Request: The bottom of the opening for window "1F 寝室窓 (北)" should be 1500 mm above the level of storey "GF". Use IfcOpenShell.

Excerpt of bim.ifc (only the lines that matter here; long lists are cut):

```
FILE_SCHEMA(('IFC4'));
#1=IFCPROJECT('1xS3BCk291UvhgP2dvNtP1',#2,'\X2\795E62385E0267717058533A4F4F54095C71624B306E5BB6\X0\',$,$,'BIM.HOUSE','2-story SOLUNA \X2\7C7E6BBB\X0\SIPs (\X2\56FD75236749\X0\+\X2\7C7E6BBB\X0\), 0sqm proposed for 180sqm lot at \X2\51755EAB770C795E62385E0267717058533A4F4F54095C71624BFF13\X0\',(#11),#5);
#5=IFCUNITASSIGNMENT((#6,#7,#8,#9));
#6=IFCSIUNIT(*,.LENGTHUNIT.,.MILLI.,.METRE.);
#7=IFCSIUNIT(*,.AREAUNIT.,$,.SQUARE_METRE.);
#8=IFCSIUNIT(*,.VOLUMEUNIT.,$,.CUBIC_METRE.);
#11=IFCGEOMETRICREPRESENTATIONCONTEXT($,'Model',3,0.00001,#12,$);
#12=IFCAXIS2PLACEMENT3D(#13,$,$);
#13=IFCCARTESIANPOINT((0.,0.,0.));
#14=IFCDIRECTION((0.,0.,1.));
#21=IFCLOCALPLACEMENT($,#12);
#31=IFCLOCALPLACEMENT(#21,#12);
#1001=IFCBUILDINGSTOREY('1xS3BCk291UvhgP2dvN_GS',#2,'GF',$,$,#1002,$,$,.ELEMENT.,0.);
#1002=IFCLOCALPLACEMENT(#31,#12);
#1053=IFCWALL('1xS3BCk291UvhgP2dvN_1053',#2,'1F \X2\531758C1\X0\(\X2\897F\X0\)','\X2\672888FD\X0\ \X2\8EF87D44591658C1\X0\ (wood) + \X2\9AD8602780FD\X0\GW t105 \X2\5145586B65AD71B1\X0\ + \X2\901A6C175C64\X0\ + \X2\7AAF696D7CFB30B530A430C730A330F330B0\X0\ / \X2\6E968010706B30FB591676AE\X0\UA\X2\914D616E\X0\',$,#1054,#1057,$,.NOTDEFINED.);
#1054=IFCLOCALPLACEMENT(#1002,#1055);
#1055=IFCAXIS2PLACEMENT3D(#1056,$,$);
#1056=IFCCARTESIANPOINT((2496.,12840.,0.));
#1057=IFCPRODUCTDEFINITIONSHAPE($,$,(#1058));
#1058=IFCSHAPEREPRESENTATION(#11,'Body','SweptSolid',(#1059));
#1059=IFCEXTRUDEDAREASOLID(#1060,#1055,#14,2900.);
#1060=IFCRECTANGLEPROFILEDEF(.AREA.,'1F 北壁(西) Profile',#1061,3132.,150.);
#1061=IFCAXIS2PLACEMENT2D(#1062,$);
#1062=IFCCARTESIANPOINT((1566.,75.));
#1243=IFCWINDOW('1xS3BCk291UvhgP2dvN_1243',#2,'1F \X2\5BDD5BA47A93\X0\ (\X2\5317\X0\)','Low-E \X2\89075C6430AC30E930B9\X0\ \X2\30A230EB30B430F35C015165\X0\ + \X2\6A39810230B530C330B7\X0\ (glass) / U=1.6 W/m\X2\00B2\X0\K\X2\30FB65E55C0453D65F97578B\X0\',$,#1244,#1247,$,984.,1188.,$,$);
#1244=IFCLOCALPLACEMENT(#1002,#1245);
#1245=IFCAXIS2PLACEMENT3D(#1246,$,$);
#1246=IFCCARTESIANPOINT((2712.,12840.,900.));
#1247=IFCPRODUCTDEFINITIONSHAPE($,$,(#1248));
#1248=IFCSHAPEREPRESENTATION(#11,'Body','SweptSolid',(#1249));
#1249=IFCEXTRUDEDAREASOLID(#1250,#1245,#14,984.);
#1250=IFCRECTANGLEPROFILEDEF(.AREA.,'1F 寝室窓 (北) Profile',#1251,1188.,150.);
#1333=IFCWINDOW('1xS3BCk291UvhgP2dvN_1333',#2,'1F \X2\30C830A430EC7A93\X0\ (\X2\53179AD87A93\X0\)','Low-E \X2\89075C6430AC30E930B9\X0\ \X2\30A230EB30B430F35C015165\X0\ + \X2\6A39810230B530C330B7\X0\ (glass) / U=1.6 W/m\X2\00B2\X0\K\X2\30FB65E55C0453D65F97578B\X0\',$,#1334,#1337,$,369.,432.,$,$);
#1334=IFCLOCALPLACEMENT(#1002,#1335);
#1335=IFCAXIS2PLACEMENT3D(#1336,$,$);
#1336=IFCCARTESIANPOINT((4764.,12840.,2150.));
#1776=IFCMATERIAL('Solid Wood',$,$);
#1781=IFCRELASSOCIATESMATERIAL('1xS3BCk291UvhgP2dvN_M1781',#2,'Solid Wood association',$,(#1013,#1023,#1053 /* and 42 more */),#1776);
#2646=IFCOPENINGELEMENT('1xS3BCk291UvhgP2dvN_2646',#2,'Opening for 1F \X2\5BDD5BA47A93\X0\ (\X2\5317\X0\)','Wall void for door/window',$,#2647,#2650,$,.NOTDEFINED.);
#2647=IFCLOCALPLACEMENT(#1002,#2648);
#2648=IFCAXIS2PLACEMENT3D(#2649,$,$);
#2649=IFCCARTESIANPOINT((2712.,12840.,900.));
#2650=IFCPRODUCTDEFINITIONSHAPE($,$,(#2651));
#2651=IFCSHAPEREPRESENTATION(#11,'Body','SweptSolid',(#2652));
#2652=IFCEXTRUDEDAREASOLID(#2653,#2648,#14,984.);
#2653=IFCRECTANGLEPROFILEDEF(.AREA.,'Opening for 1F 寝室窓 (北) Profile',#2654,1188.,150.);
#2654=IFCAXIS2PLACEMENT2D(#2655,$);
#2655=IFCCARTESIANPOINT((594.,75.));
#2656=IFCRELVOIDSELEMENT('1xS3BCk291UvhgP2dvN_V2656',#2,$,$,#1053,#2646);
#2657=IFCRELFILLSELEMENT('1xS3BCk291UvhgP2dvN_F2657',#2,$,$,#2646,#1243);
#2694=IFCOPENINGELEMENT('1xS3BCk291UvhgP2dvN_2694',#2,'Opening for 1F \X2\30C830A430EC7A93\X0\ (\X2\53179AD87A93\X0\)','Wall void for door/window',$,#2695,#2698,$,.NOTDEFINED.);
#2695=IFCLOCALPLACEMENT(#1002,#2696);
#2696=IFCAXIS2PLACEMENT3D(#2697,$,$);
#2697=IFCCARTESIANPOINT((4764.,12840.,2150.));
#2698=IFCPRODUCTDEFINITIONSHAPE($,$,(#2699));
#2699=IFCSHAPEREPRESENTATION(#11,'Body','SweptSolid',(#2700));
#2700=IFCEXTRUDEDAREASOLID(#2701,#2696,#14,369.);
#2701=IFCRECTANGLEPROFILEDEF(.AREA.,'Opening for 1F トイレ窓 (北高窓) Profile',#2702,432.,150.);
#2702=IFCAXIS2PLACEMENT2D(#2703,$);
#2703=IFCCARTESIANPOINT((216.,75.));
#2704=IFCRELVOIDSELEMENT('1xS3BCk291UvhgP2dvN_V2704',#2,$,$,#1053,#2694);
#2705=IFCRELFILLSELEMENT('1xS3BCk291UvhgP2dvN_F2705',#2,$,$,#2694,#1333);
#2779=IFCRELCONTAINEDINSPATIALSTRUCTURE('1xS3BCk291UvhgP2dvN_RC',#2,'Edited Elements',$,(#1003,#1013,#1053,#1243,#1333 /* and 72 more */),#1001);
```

```python
import numpy as np
import ifcopenshell
import ifcopenshell.api.geometry
import ifcopenshell.geom
import ifcopenshell.util.element
import ifcopenshell.util.placement
import ifcopenshell.util.shape
import ifcopenshell.util.unit

model = ifcopenshell.open("bim.ifc")
unit_scale = ifcopenshell.util.unit.calculate_unit_scale(model)

window = model.by_guid("1xS3BCk291UvhgP2dvN_1243")
opening = window.FillsVoids[0].RelatingOpeningElement
storey = ifcopenshell.util.element.get_container(window, ifc_class="IfcBuildingStorey")
level = ifcopenshell.util.placement.get_local_placement(storey.ObjectPlacement)[2, 3]

# The opening's origin need not be at the sill, so measure its lowest point.
shape = ifcopenshell.geom.create_shape(ifcopenshell.geom.settings(), opening)
bottom = ifcopenshell.util.shape.get_shape_bottom_elevation(shape, shape.geometry) / unit_scale
dz = level + 1.5 / unit_scale - bottom

shift = np.array([0.0, 0.0, dz])
# The window is not placed relative to its opening, so move both.
for product in (opening, window):
    matrix = ifcopenshell.util.placement.get_local_placement(product.ObjectPlacement)
    matrix[:3, 3] += shift
    ifcopenshell.api.geometry.edit_object_placement(model, product=product, matrix=matrix, is_si=False)

print(f"moved by {dz * unit_scale:+.3f} m")

model.write("bim-out.ifc")
```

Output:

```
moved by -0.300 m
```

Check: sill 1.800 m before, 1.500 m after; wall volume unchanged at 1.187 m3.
